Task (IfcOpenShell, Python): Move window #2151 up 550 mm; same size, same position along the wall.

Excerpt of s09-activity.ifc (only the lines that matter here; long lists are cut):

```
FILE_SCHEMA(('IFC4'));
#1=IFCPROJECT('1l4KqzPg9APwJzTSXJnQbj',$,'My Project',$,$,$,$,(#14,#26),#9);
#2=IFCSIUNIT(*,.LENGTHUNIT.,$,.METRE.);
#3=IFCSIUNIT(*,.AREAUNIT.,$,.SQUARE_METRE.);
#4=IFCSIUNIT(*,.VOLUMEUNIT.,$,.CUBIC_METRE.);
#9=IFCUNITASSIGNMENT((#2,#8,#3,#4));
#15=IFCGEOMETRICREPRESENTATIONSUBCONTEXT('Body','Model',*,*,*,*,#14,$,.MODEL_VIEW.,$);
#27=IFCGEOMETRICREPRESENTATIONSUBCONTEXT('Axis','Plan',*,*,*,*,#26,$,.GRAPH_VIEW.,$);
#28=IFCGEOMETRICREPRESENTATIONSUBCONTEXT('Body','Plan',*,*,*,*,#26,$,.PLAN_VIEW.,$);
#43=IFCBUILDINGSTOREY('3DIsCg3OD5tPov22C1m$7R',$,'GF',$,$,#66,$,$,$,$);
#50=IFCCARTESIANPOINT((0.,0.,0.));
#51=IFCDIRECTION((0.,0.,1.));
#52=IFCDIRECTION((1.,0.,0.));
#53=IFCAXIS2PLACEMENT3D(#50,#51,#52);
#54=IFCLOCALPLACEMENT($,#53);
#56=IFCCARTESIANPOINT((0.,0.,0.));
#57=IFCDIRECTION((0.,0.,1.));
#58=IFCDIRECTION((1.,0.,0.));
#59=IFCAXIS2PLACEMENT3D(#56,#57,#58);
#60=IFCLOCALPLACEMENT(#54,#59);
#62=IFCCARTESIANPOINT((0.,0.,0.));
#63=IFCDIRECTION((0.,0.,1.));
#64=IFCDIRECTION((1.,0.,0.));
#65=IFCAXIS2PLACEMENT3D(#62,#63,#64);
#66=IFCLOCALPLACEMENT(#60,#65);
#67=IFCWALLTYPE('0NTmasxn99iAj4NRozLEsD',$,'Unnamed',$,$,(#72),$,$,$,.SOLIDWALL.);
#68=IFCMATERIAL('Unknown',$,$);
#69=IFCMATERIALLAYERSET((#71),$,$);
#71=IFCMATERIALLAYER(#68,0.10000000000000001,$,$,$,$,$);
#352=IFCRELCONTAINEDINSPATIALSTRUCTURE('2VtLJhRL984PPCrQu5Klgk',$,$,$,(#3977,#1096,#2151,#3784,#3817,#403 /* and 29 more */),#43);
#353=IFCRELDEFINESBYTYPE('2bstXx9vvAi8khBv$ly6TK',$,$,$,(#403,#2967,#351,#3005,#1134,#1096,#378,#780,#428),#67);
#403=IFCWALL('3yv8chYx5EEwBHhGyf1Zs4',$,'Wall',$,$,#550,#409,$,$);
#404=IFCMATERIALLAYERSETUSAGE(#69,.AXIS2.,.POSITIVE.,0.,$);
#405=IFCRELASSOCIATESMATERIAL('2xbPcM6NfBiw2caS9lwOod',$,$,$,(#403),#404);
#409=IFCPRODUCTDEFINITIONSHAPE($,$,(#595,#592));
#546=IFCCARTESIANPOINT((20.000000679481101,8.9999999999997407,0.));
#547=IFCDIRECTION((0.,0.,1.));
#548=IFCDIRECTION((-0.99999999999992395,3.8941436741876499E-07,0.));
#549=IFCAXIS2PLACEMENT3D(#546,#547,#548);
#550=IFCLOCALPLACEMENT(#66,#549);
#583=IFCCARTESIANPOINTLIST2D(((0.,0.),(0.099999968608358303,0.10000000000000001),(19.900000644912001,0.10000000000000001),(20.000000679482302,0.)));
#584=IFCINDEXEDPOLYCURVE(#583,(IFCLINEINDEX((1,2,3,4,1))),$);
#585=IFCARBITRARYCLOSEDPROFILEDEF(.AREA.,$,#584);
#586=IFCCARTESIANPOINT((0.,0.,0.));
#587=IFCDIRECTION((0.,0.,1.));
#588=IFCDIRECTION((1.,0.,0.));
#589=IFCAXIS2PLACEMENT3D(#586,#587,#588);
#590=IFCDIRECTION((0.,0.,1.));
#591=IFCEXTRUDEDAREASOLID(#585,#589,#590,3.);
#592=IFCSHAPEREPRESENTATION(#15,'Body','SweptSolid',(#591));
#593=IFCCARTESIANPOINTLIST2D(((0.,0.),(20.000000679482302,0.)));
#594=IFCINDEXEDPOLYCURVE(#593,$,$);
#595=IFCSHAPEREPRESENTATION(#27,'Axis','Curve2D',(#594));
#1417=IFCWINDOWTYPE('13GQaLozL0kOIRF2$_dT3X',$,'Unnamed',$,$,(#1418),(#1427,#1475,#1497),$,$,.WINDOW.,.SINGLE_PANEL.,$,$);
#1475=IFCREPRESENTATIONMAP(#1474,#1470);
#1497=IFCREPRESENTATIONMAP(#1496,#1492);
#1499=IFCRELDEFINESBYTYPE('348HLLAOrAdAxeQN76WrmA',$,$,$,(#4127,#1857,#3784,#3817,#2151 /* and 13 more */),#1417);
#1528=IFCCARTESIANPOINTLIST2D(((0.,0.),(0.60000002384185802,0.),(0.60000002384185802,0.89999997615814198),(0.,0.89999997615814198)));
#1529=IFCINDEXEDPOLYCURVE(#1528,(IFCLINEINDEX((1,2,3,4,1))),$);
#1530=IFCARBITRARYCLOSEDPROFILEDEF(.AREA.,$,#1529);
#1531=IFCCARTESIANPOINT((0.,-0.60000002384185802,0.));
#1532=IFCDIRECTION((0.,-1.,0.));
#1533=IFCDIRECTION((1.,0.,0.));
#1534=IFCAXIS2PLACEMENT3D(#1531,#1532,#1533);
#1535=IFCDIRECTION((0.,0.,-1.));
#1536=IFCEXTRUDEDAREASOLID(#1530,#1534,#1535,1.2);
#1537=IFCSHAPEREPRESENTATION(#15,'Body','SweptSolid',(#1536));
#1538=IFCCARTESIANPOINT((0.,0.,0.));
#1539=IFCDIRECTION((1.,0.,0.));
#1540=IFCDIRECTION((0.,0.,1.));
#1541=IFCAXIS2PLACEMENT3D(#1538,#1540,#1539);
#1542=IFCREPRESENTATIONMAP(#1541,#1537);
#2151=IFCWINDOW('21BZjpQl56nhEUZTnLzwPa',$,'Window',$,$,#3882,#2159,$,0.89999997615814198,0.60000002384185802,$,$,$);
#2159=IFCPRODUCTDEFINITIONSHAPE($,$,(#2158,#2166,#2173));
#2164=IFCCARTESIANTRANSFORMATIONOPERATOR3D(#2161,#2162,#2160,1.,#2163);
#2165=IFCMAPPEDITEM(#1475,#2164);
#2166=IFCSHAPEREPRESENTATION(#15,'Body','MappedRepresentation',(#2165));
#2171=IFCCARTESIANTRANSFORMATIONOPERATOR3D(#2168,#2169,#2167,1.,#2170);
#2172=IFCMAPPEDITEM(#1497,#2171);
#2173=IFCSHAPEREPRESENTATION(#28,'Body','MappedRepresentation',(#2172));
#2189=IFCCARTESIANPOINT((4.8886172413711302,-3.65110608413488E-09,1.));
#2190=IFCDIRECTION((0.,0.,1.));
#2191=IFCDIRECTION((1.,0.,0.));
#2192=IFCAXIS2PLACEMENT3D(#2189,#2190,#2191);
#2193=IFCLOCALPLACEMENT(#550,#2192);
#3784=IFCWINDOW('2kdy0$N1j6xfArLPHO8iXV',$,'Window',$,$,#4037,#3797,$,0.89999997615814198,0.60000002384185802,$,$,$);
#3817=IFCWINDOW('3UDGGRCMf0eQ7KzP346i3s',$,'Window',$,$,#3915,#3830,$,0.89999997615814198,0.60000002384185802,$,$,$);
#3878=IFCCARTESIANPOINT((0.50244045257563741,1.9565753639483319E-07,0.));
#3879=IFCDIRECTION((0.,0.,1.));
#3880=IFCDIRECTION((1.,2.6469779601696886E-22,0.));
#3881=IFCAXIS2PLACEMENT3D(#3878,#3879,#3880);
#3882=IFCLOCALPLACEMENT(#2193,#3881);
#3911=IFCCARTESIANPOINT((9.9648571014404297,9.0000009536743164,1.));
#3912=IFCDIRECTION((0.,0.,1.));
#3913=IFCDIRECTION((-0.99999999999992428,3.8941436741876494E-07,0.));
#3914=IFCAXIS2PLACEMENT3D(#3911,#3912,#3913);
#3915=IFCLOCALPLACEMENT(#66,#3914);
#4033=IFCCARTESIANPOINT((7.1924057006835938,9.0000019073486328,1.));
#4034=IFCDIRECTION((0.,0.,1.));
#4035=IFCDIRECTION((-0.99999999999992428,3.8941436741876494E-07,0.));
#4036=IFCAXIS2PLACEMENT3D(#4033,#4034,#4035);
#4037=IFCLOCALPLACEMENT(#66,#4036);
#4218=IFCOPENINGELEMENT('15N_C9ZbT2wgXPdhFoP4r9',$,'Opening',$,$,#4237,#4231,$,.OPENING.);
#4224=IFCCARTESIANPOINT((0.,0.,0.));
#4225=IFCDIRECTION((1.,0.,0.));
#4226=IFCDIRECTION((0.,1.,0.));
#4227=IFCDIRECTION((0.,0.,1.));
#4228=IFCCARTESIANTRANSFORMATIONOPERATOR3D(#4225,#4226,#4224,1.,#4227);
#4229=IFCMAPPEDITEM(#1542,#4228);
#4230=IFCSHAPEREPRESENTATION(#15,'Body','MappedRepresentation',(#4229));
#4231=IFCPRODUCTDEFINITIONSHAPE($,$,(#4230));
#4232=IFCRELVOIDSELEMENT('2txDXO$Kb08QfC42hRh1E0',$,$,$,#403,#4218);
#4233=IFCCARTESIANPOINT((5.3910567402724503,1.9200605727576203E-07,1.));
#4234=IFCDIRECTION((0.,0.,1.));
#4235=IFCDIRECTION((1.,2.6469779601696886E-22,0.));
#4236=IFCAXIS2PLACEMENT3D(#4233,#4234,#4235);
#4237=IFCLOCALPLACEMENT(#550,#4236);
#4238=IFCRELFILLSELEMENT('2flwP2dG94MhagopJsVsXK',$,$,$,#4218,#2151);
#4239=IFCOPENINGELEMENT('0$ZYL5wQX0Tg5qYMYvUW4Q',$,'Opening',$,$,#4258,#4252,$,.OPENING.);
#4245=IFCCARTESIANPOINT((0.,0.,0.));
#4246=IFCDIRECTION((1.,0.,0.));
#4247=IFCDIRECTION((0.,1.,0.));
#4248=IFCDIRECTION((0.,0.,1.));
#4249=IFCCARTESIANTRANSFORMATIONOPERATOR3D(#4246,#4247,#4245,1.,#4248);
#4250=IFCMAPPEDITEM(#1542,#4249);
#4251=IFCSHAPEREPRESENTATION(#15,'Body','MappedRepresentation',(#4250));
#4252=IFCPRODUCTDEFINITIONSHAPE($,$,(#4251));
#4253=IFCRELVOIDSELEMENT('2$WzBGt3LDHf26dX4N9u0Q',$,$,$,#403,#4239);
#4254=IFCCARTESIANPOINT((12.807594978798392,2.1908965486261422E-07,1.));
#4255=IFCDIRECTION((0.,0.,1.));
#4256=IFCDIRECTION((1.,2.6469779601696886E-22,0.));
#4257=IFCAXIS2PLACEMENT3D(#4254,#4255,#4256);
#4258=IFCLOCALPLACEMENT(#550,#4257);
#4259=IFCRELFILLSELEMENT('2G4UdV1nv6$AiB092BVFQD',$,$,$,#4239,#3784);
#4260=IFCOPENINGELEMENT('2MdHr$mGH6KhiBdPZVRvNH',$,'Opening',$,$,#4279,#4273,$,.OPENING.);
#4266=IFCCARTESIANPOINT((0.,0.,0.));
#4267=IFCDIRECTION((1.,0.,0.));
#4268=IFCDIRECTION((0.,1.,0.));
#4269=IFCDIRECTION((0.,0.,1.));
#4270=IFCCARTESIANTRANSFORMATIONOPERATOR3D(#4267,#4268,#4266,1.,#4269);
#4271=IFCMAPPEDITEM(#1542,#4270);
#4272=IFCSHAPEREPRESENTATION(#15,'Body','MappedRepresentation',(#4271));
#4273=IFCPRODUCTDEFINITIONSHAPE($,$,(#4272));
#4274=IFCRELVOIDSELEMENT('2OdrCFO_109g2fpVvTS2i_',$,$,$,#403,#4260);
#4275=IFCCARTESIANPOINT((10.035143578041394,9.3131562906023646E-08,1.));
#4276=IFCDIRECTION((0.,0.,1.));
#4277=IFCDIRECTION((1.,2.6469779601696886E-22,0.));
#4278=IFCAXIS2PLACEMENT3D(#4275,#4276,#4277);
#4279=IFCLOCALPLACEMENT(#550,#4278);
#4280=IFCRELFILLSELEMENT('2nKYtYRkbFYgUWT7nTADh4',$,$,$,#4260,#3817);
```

```python
import numpy as np
import ifcopenshell
import ifcopenshell.api.geometry
import ifcopenshell.util.placement
import ifcopenshell.util.unit

model = ifcopenshell.open("s09-activity.ifc")
unit_scale = ifcopenshell.util.unit.calculate_unit_scale(model)

window = model.by_guid("21BZjpQl56nhEUZTnLzwPa")
opening = window.FillsVoids[0].RelatingOpeningElement
dz = 0.55

shift = np.array([0.0, 0.0, dz])
# The window is not placed relative to its opening, so move both.
for product in (opening, window):
    matrix = ifcopenshell.util.placement.get_local_placement(product.ObjectPlacement)
    matrix[:3, 3] += shift
    ifcopenshell.api.geometry.edit_object_placement(model, product=product, matrix=matrix, is_si=False)

print(f"moved by {dz * unit_scale:+.3f} m")

model.write("s09-activity_rev.ifc")
```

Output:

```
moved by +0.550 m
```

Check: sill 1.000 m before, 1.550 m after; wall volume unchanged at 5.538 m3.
